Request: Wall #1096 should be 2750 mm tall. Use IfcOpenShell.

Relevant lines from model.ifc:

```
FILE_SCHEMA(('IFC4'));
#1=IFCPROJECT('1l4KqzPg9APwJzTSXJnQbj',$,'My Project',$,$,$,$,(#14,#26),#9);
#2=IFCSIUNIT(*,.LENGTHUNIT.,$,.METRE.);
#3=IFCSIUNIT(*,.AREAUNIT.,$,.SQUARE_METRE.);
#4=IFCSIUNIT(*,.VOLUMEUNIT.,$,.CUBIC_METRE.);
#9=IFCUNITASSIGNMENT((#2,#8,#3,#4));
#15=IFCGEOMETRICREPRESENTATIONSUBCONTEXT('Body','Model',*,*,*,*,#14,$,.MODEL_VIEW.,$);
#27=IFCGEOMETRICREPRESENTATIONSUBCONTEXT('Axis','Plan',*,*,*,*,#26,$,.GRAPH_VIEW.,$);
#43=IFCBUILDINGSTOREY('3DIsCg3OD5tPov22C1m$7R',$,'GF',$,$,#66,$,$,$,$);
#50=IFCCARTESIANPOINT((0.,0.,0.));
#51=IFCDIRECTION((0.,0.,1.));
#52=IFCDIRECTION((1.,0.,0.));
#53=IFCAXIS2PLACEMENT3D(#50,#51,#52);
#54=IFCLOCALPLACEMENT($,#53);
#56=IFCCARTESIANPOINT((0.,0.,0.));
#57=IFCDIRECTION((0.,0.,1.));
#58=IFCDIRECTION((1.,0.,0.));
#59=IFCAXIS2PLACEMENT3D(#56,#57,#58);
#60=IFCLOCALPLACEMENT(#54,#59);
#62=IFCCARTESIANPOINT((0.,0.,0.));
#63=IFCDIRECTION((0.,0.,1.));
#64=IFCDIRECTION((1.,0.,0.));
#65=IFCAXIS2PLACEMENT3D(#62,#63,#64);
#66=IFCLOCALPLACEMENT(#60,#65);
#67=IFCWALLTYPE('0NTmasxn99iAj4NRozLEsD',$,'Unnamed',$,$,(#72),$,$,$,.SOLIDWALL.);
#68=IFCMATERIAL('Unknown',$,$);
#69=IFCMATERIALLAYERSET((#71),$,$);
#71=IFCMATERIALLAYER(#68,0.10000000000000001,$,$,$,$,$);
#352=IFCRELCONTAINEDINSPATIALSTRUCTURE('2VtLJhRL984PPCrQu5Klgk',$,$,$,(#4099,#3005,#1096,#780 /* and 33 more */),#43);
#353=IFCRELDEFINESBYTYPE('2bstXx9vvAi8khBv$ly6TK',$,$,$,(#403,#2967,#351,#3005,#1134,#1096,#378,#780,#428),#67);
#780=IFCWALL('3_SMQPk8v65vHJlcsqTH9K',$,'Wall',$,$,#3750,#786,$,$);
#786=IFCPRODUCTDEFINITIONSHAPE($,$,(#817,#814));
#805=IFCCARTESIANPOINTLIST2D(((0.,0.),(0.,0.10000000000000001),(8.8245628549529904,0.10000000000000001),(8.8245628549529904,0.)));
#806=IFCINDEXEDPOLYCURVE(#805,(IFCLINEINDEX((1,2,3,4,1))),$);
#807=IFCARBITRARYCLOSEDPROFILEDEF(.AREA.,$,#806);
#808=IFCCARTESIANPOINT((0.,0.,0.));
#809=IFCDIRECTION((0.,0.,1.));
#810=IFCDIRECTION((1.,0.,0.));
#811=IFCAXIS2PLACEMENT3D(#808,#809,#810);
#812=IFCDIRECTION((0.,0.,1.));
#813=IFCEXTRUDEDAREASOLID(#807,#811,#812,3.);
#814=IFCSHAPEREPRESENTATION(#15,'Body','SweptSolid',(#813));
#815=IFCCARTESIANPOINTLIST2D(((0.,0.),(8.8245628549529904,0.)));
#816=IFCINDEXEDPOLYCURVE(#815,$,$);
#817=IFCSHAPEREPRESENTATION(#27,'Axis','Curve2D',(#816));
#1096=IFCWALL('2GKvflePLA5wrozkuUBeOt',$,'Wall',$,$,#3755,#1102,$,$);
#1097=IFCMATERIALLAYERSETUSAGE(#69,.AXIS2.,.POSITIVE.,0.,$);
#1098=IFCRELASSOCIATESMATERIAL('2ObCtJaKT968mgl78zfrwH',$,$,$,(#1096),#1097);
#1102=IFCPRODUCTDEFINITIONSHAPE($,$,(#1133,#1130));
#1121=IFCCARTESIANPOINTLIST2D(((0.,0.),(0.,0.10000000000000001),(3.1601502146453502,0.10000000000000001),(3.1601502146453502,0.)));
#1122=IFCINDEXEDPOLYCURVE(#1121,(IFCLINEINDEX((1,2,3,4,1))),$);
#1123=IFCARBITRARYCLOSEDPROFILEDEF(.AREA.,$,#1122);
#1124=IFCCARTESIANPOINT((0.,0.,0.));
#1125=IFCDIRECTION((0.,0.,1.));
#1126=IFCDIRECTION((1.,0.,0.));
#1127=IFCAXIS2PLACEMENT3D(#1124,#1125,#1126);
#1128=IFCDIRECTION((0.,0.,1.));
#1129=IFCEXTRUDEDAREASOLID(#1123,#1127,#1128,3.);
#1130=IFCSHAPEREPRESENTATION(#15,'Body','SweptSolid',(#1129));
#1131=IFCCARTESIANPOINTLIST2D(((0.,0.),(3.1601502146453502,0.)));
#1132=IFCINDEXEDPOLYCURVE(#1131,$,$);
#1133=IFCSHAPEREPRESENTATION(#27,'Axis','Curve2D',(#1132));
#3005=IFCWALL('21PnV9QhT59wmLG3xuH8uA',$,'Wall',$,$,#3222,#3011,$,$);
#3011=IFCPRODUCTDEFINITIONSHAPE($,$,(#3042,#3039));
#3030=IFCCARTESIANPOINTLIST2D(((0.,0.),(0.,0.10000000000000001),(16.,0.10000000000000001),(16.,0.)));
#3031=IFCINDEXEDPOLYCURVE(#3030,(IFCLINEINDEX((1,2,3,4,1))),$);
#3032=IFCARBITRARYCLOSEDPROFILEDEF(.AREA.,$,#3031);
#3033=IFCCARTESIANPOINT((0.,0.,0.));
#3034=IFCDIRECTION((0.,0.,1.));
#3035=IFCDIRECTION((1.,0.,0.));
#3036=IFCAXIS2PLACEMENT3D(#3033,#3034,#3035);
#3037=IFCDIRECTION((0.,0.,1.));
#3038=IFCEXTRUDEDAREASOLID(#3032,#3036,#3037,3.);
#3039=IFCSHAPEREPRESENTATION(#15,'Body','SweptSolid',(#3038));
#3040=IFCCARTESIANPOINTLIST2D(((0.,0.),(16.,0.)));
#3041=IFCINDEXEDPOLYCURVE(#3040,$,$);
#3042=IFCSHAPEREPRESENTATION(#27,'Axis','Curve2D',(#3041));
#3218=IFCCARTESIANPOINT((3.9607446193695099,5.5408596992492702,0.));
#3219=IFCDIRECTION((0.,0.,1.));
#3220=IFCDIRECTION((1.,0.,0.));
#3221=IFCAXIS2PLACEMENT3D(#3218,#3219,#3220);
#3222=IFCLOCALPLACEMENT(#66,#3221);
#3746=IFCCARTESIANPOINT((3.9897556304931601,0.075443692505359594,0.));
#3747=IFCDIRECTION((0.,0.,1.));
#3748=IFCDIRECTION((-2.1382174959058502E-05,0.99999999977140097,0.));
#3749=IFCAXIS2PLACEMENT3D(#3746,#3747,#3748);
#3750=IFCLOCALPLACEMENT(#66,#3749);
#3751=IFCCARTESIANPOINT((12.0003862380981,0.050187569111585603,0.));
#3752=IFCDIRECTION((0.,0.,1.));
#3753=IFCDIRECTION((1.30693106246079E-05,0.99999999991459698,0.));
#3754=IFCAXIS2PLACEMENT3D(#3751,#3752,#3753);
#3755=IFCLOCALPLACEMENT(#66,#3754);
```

```python
import ifcopenshell
import ifcopenshell.geom
import ifcopenshell.util.representation
import ifcopenshell.util.shape
import ifcopenshell.util.unit

model = ifcopenshell.open("model.ifc")
unit_scale = ifcopenshell.util.unit.calculate_unit_scale(model)
settings = ifcopenshell.geom.settings()


def volume(element):
    """Net volume in cubic metres, openings subtracted."""
    shape = ifcopenshell.geom.create_shape(settings, element)
    return ifcopenshell.util.shape.get_volume(shape.geometry)


wall = model.by_guid("2GKvflePLA5wrozkuUBeOt")
before = volume(wall)

body = ifcopenshell.util.representation.get_representation(wall, "Model", "Body")
solid = body.Items[0]
old_height = solid.Depth
solid.Depth = 2.75 / unit_scale
after = volume(wall)

print(f"height {old_height:g} -> {solid.Depth:g}, volume {before:.3f} -> {after:.3f} m3")

model.write("model_edited.ifc")
```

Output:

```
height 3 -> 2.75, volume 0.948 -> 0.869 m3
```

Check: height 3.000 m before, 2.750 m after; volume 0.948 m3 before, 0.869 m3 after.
